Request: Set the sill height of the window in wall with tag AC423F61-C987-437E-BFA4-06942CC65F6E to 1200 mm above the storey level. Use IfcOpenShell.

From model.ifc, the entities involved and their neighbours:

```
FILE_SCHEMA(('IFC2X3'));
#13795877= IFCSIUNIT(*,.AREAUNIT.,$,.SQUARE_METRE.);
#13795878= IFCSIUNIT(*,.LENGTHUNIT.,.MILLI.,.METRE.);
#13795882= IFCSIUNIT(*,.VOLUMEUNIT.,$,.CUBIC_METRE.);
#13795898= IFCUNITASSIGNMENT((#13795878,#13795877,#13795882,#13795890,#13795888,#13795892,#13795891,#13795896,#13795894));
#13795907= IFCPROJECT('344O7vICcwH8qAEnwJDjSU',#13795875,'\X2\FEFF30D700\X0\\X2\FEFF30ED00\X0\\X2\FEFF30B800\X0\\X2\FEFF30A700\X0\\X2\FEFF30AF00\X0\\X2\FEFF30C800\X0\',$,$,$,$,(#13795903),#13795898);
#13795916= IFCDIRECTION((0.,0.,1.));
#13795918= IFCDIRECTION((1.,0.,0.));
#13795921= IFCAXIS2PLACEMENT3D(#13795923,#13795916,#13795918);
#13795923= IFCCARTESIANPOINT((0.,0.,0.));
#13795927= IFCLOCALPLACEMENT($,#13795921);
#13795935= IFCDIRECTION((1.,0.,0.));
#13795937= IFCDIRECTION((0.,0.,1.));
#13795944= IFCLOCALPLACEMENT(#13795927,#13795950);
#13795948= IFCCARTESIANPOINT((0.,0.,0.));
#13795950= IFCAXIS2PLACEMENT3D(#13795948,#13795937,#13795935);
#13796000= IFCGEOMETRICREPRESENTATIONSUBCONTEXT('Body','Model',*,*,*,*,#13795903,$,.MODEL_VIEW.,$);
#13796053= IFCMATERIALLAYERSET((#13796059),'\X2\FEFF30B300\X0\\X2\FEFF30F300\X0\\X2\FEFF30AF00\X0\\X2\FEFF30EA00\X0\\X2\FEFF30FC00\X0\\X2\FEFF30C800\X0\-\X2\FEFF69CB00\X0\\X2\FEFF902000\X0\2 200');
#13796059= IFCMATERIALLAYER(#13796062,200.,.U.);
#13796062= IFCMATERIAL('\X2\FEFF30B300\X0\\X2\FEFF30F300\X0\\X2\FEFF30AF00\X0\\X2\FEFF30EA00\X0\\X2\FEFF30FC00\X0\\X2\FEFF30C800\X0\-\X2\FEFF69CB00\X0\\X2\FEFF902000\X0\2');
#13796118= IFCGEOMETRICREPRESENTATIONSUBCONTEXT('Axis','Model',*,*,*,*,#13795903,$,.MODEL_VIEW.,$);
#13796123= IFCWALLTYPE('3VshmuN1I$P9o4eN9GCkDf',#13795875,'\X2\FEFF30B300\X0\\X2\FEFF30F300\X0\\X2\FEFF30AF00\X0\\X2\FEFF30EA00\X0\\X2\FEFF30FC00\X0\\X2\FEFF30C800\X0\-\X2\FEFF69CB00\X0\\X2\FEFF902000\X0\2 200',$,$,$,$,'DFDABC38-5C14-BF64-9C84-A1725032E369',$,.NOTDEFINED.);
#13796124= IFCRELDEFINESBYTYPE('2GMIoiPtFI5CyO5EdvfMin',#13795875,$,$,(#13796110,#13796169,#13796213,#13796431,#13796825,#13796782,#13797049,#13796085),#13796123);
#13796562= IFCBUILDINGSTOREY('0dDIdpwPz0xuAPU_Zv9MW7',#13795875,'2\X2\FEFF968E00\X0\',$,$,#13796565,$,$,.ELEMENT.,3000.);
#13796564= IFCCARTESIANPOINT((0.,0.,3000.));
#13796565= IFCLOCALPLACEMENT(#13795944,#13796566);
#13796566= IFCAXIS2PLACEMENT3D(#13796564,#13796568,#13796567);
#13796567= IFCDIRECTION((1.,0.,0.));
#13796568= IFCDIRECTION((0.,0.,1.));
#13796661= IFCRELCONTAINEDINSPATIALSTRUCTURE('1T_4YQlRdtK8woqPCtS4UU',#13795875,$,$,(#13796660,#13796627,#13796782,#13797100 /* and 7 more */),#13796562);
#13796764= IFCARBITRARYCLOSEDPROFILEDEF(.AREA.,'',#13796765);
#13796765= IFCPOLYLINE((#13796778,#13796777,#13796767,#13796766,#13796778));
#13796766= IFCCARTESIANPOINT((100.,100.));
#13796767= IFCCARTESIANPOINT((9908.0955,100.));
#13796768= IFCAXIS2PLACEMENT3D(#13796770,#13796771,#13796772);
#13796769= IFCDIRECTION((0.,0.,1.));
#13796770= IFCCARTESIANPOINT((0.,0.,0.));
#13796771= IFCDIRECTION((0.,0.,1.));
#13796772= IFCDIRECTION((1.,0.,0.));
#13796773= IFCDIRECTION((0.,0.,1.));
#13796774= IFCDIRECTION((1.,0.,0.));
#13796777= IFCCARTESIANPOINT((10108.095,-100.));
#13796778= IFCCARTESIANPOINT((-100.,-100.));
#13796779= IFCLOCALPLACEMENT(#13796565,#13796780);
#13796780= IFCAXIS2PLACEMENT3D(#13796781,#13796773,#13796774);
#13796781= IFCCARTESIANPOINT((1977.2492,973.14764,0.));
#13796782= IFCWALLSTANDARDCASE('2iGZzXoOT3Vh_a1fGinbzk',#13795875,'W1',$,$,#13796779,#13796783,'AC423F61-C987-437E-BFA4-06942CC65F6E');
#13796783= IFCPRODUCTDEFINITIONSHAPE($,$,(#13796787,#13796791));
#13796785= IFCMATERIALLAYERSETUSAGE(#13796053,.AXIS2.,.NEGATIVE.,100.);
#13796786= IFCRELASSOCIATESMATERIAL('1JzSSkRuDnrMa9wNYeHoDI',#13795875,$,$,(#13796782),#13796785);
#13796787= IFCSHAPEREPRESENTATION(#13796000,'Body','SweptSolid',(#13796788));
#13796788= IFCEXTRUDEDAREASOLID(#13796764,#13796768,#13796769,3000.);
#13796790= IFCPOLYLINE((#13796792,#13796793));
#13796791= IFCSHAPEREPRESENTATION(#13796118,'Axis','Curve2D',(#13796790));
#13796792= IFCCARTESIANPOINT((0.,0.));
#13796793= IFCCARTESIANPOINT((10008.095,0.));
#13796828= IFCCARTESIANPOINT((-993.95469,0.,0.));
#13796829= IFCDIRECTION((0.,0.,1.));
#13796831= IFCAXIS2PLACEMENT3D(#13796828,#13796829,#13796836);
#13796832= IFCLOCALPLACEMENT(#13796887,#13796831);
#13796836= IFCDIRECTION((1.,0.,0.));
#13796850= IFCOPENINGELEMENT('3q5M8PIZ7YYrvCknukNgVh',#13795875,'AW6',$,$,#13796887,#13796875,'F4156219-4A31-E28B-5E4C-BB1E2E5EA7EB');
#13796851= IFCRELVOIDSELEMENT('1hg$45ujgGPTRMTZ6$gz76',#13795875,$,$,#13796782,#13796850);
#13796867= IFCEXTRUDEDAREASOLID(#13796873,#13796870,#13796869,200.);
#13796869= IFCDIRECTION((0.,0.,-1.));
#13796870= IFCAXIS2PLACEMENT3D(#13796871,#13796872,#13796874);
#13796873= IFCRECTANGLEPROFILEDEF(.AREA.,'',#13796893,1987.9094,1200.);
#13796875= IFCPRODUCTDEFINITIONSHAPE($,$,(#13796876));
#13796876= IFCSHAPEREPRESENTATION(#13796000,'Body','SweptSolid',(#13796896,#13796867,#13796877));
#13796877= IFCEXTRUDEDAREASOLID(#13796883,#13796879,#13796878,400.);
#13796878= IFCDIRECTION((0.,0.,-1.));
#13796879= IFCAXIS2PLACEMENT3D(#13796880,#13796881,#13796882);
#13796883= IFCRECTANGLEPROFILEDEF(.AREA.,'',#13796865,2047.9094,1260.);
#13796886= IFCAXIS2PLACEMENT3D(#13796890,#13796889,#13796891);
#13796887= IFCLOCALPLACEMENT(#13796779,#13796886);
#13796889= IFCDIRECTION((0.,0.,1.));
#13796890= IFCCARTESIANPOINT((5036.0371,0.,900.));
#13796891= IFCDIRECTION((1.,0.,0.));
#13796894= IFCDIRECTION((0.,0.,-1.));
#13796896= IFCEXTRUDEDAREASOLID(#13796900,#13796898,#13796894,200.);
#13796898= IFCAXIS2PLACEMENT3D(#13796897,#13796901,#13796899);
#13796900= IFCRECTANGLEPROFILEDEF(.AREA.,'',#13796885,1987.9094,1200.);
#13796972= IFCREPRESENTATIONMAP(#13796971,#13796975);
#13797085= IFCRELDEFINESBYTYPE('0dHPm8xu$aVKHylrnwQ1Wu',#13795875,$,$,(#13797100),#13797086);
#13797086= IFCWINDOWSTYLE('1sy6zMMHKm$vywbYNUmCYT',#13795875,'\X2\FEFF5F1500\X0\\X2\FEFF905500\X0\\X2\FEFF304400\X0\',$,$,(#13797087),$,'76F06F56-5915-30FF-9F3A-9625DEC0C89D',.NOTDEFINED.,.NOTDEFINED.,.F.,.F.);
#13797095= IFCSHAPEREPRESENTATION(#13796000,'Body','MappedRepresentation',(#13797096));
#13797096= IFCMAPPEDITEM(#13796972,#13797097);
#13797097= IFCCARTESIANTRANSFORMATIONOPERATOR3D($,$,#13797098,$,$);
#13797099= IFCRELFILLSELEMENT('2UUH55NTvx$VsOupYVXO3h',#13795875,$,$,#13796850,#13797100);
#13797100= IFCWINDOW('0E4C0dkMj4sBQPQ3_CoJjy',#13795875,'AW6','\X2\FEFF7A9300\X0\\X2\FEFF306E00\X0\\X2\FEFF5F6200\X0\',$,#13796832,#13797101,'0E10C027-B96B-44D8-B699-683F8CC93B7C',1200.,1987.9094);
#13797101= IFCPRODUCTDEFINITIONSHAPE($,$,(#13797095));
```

```python
import numpy as np
import ifcopenshell
import ifcopenshell.api.geometry
import ifcopenshell.geom
import ifcopenshell.util.element
import ifcopenshell.util.placement
import ifcopenshell.util.shape
import ifcopenshell.util.unit

model = ifcopenshell.open("model.ifc")
unit_scale = ifcopenshell.util.unit.calculate_unit_scale(model)

window = model.by_guid("0E4C0dkMj4sBQPQ3_CoJjy")
opening = window.FillsVoids[0].RelatingOpeningElement
storey = ifcopenshell.util.element.get_container(window, ifc_class="IfcBuildingStorey")
level = ifcopenshell.util.placement.get_local_placement(storey.ObjectPlacement)[2, 3]

# The opening's origin need not be at the sill, so measure its lowest point.
shape = ifcopenshell.geom.create_shape(ifcopenshell.geom.settings(), opening)
bottom = ifcopenshell.util.shape.get_shape_bottom_elevation(shape, shape.geometry) / unit_scale
dz = level + 1.2 / unit_scale - bottom

shift = np.array([0.0, 0.0, dz])
# The window is placed relative to its opening, so it follows when the opening moves.
matrix = ifcopenshell.util.placement.get_local_placement(opening.ObjectPlacement)
matrix[:3, 3] += shift
ifcopenshell.api.geometry.edit_object_placement(
    model, product=opening, matrix=matrix, is_si=False, should_transform_children=True
)

print(f"moved by {dz * unit_scale:+.3f} m")

model.write("model_updated.ifc")
```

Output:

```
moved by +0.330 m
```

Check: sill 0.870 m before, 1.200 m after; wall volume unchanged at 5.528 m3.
